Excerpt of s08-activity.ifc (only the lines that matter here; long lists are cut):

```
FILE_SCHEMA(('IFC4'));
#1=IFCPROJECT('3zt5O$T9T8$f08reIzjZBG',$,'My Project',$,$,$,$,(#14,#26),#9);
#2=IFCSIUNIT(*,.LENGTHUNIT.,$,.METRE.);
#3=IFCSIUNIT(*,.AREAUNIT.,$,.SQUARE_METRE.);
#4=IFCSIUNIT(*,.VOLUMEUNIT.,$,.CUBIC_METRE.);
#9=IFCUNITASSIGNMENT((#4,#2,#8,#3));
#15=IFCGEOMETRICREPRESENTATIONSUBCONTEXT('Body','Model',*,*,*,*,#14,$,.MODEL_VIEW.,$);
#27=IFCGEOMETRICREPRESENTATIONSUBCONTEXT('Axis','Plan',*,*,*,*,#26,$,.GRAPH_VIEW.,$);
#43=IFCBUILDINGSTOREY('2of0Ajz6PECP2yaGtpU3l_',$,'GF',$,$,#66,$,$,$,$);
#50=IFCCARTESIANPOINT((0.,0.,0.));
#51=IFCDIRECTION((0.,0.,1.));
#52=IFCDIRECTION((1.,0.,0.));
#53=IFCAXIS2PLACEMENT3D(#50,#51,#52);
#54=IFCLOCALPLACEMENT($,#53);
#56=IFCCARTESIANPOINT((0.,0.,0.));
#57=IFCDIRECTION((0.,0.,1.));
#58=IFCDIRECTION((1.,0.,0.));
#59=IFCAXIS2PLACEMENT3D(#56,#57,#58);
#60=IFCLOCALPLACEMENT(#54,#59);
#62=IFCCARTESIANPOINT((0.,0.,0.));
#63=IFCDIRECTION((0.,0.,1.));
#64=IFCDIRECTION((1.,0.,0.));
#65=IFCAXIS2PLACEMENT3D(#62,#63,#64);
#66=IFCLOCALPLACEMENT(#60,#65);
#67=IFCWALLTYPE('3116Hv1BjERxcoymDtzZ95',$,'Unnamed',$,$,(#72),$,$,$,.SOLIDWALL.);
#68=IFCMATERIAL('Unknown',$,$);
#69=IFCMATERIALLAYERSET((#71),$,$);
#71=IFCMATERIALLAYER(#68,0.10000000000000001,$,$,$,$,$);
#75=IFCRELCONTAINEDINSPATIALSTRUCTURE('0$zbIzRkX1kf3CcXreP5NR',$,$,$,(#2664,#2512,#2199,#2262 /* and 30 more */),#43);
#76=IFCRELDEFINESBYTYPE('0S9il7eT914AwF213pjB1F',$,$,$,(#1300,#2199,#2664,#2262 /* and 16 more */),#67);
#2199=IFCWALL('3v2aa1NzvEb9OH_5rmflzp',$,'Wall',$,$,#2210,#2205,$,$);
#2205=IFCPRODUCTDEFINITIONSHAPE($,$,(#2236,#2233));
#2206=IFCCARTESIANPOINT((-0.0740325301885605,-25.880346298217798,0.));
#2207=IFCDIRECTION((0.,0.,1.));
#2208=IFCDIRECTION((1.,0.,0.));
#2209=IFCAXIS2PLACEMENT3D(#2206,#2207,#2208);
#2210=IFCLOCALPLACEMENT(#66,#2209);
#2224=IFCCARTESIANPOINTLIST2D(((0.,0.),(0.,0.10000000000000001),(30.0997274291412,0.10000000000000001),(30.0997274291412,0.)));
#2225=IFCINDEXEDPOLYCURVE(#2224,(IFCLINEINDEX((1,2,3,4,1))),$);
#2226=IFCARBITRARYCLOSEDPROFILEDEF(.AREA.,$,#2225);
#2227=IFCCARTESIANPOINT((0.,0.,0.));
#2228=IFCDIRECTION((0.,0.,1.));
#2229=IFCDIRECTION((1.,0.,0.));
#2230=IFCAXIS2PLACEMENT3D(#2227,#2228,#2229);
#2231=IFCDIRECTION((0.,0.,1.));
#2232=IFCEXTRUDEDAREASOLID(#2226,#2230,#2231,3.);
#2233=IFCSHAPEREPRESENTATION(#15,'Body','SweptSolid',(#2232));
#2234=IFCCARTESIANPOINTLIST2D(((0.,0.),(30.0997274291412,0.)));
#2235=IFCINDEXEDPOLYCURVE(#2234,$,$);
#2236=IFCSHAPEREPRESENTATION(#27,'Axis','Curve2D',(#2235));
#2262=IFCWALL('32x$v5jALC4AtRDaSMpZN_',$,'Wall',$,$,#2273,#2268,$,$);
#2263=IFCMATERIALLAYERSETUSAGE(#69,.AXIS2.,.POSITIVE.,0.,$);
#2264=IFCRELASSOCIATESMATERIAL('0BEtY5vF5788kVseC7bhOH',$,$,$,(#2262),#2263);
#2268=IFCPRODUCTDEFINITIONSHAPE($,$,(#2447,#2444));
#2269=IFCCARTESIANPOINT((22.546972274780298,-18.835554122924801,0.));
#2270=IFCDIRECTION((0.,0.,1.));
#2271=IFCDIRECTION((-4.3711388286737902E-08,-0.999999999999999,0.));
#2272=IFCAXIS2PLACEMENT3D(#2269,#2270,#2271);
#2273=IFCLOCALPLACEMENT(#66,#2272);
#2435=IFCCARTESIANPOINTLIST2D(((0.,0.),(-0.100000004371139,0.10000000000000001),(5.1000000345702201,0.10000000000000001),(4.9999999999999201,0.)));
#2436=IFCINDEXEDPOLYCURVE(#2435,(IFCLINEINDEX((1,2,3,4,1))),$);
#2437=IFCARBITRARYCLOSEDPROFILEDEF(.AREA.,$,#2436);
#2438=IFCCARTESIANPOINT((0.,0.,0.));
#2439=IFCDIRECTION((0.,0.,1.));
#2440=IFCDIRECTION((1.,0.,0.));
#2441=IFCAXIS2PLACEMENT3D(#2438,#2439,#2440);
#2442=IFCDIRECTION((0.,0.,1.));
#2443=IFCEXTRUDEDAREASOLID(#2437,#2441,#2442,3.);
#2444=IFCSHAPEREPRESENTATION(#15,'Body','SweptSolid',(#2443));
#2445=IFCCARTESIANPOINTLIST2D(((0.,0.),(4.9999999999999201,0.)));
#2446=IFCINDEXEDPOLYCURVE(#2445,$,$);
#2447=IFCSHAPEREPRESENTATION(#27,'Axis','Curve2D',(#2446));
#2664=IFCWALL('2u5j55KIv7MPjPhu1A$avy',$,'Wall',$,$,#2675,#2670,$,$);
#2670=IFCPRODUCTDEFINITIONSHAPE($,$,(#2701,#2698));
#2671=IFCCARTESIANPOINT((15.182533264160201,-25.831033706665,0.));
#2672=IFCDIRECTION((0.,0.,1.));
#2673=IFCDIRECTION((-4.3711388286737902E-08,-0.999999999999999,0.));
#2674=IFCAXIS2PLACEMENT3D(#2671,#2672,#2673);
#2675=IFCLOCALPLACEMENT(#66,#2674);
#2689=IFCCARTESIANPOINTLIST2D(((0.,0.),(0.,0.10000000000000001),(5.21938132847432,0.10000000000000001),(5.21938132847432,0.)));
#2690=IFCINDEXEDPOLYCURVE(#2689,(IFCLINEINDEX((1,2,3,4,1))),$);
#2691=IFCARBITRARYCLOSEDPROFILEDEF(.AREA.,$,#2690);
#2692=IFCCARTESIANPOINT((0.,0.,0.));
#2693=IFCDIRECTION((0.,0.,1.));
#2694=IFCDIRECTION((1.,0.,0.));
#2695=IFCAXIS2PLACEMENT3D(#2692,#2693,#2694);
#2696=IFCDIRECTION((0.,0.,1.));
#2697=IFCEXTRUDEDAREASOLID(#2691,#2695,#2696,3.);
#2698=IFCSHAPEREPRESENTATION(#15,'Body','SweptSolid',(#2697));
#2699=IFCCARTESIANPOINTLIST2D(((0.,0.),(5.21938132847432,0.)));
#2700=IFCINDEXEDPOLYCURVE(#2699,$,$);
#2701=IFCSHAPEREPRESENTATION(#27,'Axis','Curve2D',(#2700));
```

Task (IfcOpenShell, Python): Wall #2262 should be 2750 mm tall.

```python
import ifcopenshell
import ifcopenshell.geom
import ifcopenshell.util.representation
import ifcopenshell.util.shape
import ifcopenshell.util.unit

model = ifcopenshell.open("s08-activity.ifc")
unit_scale = ifcopenshell.util.unit.calculate_unit_scale(model)
settings = ifcopenshell.geom.settings()


def volume(element):
    """Net volume in cubic metres, openings subtracted."""
    shape = ifcopenshell.geom.create_shape(settings, element)
    return ifcopenshell.util.shape.get_volume(shape.geometry)


wall = model.by_guid("32x$v5jALC4AtRDaSMpZN_")
before = volume(wall)

body = ifcopenshell.util.representation.get_representation(wall, "Model", "Body")
solid = body.Items[0]
old_height = solid.Depth
solid.Depth = 2.75 / unit_scale
after = volume(wall)

print(f"height {old_height:g} -> {solid.Depth:g}, volume {before:.3f} -> {after:.3f} m3")

model.write("s08-activity_rev.ifc")
```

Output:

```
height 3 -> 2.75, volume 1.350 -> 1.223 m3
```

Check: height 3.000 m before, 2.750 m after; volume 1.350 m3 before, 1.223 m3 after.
